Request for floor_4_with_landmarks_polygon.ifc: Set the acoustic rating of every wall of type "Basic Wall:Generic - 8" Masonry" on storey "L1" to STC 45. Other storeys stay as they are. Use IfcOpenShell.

First a look at what the model holds.

```python
import ifcopenshell
import ifcopenshell.util.element

model = ifcopenshell.open("floor_4_with_landmarks_polygon.ifc")
print(model.schema)
storey = next(s for s in model.by_type("IfcBuildingStorey") if s.Name == "L1")
walls = [e for e in ifcopenshell.util.element.get_decomposition(storey) if e.is_a("IfcWall")]
seen = {}
for e in walls:
    element_type = ifcopenshell.util.element.get_type(e)
    key = (element_type.Name if element_type != e and element_type else None, ifcopenshell.util.element.get_pset(e, "Pset_WallCommon", "AcousticRating"))
    seen[key] = seen.get(key, 0) + 1
for (name, value), count in sorted(seen.items(), key=str):
    print(count, "x", name, "|", value)
```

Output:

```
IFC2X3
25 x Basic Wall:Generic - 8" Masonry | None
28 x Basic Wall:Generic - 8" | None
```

```python
import ifcopenshell
import ifcopenshell.api.pset
import ifcopenshell.util.element

model = ifcopenshell.open("floor_4_with_landmarks_polygon.ifc")

storey = next(s for s in model.by_type("IfcBuildingStorey") if s.Name == "L1")
walls = [e for e in ifcopenshell.util.element.get_decomposition(storey) if e.is_a("IfcWall")]

count = 0
for e in walls:
    element_type = ifcopenshell.util.element.get_type(e)
    if element_type in (None, e) or element_type.Name != 'Basic Wall:Generic - 8" Masonry':
        continue
    # add_pset returns the element's existing set when there is one.
    pset = ifcopenshell.api.pset.add_pset(model, product=e, name="Pset_WallCommon")
    ifcopenshell.api.pset.edit_pset(model, pset=pset, properties={"AcousticRating": "STC 45"})
    count += 1

print(count, "walls updated")

model.write("floor_4_with_landmarks_polygon-out.ifc")
```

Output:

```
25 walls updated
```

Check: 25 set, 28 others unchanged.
